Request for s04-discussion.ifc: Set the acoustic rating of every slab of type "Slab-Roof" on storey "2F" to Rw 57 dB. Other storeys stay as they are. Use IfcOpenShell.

First a look at what the model holds.

```python
import ifcopenshell
import ifcopenshell.util.element

model = ifcopenshell.open("s04-discussion.ifc")
print(model.schema)
storey = next(s for s in model.by_type("IfcBuildingStorey") if s.Name == "2F")
slabs = [e for e in ifcopenshell.util.element.get_decomposition(storey) if e.is_a("IfcSlab")]
seen = {}
for e in slabs:
    element_type = ifcopenshell.util.element.get_type(e)
    key = (element_type.Name if element_type != e and element_type else None, ifcopenshell.util.element.get_pset(e, "Pset_SlabCommon", "AcousticRating"))
    seen[key] = seen.get(key, 0) + 1
for (name, value), count in sorted(seen.items(), key=str):
    print(count, "x", name, "|", value)
```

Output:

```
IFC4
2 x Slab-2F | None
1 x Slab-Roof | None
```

```python
import ifcopenshell
import ifcopenshell.api.pset
import ifcopenshell.util.element

model = ifcopenshell.open("s04-discussion.ifc")

storey = next(s for s in model.by_type("IfcBuildingStorey") if s.Name == "2F")
slabs = [e for e in ifcopenshell.util.element.get_decomposition(storey) if e.is_a("IfcSlab")]

count = 0
for e in slabs:
    element_type = ifcopenshell.util.element.get_type(e)
    if element_type in (None, e) or element_type.Name != "Slab-Roof":
        continue
    # add_pset returns the element's existing set when there is one.
    pset = ifcopenshell.api.pset.add_pset(model, product=e, name="Pset_SlabCommon")
    ifcopenshell.api.pset.edit_pset(model, pset=pset, properties={"AcousticRating": "Rw 57 dB"})
    count += 1

print(count, "slabs updated")

model.write("s04-discussion_rev.ifc")
```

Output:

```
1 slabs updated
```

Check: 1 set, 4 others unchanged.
